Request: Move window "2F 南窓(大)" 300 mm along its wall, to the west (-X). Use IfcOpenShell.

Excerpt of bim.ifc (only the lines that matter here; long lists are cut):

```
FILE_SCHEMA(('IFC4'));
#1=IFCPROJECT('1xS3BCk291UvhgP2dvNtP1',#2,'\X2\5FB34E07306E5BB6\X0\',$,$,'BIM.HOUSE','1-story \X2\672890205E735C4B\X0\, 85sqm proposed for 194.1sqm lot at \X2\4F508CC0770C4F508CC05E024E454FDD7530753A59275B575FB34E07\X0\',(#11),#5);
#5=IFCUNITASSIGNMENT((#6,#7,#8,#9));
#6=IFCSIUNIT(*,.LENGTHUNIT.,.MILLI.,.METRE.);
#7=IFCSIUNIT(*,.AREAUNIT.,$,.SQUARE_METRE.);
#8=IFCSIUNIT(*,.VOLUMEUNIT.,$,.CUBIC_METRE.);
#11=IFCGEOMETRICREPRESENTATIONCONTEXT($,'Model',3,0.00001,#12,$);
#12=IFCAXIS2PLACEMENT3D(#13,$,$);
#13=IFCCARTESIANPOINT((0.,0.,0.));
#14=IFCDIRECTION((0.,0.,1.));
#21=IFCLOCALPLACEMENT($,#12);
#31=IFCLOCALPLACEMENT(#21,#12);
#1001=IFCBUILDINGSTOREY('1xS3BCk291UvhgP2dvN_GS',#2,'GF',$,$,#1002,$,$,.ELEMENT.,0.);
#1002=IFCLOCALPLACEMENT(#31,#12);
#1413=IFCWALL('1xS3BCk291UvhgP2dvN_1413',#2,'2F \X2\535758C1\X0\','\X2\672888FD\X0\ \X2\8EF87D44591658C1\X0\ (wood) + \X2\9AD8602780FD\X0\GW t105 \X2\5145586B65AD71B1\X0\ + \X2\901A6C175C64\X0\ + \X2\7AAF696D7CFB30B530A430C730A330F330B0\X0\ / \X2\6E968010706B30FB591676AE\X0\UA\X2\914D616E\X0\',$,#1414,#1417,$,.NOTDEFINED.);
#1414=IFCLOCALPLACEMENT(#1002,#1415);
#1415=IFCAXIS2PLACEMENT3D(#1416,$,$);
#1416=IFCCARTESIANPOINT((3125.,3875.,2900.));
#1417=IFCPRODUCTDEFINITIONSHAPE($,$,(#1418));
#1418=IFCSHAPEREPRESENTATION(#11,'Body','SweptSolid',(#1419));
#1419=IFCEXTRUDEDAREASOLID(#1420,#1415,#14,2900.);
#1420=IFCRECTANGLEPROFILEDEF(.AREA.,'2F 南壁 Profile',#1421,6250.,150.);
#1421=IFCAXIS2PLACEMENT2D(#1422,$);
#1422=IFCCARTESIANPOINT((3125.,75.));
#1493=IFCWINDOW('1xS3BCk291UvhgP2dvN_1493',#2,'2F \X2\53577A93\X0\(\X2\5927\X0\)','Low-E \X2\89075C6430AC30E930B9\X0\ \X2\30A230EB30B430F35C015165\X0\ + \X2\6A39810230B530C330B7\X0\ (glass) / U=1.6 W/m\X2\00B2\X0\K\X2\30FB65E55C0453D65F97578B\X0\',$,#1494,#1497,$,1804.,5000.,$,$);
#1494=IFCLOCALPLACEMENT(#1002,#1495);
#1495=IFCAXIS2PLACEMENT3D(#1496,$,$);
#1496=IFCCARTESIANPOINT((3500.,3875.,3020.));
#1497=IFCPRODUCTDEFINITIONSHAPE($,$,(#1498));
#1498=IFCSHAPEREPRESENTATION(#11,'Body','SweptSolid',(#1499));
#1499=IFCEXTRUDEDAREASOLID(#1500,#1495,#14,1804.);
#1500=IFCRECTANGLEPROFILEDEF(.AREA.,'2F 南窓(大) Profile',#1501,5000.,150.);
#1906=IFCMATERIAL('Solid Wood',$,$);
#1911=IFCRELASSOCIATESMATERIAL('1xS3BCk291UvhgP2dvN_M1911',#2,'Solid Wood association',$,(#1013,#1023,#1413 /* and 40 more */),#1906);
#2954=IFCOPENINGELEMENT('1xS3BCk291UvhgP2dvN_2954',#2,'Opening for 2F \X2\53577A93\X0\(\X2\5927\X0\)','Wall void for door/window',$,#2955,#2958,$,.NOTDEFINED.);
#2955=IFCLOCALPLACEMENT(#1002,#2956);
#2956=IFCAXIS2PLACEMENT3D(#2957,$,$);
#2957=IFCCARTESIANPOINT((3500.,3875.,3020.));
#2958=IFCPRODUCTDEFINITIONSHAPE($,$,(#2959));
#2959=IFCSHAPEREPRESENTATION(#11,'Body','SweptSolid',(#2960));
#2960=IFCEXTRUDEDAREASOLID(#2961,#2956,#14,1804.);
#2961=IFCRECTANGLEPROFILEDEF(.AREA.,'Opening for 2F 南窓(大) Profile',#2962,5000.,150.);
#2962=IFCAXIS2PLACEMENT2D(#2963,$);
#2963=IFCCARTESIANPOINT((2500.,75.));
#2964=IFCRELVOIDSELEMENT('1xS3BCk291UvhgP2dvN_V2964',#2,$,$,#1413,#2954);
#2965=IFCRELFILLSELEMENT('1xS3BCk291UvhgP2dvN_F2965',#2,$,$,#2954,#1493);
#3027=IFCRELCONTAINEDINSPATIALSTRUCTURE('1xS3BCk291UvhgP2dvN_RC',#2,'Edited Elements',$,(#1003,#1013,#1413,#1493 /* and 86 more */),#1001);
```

```python
import ifcopenshell
import ifcopenshell.api.geometry
import ifcopenshell.util.placement
import ifcopenshell.util.unit

model = ifcopenshell.open("bim.ifc")
unit_scale = ifcopenshell.util.unit.calculate_unit_scale(model)

window = model.by_guid("1xS3BCk291UvhgP2dvN_1493")
opening = window.FillsVoids[0].RelatingOpeningElement
wall = opening.VoidsElements[0].RelatingBuildingElement

wall_matrix = ifcopenshell.util.placement.get_local_placement(wall.ObjectPlacement)
shift = wall_matrix[:3, 0] * -0.3 / unit_scale
before = ifcopenshell.util.placement.get_local_placement(window.ObjectPlacement)[:3, 3].copy()

# The window is not placed relative to its opening, so move both.
for product in (opening, window):
    matrix = ifcopenshell.util.placement.get_local_placement(product.ObjectPlacement)
    matrix[:3, 3] += shift
    ifcopenshell.api.geometry.edit_object_placement(model, product=product, matrix=matrix, is_si=False)

after = ifcopenshell.util.placement.get_local_placement(window.ObjectPlacement)[:3, 3]
print("window moved by", (after - before).round(3) + 0.0)

model.write("bim_edited.ifc")
```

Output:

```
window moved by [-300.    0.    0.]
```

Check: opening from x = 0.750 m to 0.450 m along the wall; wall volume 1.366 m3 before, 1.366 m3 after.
